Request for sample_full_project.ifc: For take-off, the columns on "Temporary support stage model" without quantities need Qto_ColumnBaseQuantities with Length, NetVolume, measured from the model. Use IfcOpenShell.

First a look at what the model holds.

```python
import ifcopenshell
import ifcopenshell.util.element
import ifcopenshell.util.unit

model = ifcopenshell.open("sample_full_project.ifc")
print(model.schema)
for unit_type in ("LENGTHUNIT", "AREAUNIT", "VOLUMEUNIT"):
    print(unit_type, ifcopenshell.util.unit.calculate_unit_scale(model, unit_type))
storey = next(s for s in model.by_type("IfcBuildingStorey") if s.Name == "Temporary support stage model")
columns = [e for e in ifcopenshell.util.element.get_decomposition(storey) if e.is_a("IfcColumn")]
for e in sorted(columns, key=lambda e: e.id()):
    print(e.id(), e.is_a(), e.Name, list(ifcopenshell.util.element.get_psets(e, qtos_only=True)), sep=" | ")
```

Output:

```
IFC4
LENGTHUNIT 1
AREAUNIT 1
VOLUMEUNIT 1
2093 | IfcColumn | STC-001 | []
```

```python
import ifcopenshell
import ifcopenshell.api.pset
import ifcopenshell.geom
import ifcopenshell.util.element
import ifcopenshell.util.shape
import ifcopenshell.util.unit

model = ifcopenshell.open("sample_full_project.ifc")
unit_scale = ifcopenshell.util.unit.calculate_unit_scale(model)
volume_scale = ifcopenshell.util.unit.calculate_unit_scale(model, "VOLUMEUNIT")
settings = ifcopenshell.geom.settings()

storey = next(s for s in model.by_type("IfcBuildingStorey") if s.Name == "Temporary support stage model")
columns = [e for e in ifcopenshell.util.element.get_decomposition(storey) if e.is_a("IfcColumn")]

for e in sorted(columns, key=lambda e: e.id()):
    if ifcopenshell.util.element.get_psets(e, qtos_only=True, should_inherit=False):
        continue
    # Geometry comes back in metres, in the element's own axes.
    shape = ifcopenshell.geom.create_shape(settings, e)
    values = {
        "Length": ifcopenshell.util.shape.get_z(shape.geometry) / unit_scale,
        "NetVolume": ifcopenshell.util.shape.get_volume(shape.geometry) / volume_scale,
    }
    qto = ifcopenshell.api.pset.add_qto(model, product=e, name="Qto_ColumnBaseQuantities")
    ifcopenshell.api.pset.edit_qto(model, qto=qto, properties=values)
    print(e.id(), {k: round(v, 3) for k, v in values.items()})

model.write("sample_full_project-out.ifc")
```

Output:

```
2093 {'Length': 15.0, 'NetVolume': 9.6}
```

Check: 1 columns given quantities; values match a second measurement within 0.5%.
